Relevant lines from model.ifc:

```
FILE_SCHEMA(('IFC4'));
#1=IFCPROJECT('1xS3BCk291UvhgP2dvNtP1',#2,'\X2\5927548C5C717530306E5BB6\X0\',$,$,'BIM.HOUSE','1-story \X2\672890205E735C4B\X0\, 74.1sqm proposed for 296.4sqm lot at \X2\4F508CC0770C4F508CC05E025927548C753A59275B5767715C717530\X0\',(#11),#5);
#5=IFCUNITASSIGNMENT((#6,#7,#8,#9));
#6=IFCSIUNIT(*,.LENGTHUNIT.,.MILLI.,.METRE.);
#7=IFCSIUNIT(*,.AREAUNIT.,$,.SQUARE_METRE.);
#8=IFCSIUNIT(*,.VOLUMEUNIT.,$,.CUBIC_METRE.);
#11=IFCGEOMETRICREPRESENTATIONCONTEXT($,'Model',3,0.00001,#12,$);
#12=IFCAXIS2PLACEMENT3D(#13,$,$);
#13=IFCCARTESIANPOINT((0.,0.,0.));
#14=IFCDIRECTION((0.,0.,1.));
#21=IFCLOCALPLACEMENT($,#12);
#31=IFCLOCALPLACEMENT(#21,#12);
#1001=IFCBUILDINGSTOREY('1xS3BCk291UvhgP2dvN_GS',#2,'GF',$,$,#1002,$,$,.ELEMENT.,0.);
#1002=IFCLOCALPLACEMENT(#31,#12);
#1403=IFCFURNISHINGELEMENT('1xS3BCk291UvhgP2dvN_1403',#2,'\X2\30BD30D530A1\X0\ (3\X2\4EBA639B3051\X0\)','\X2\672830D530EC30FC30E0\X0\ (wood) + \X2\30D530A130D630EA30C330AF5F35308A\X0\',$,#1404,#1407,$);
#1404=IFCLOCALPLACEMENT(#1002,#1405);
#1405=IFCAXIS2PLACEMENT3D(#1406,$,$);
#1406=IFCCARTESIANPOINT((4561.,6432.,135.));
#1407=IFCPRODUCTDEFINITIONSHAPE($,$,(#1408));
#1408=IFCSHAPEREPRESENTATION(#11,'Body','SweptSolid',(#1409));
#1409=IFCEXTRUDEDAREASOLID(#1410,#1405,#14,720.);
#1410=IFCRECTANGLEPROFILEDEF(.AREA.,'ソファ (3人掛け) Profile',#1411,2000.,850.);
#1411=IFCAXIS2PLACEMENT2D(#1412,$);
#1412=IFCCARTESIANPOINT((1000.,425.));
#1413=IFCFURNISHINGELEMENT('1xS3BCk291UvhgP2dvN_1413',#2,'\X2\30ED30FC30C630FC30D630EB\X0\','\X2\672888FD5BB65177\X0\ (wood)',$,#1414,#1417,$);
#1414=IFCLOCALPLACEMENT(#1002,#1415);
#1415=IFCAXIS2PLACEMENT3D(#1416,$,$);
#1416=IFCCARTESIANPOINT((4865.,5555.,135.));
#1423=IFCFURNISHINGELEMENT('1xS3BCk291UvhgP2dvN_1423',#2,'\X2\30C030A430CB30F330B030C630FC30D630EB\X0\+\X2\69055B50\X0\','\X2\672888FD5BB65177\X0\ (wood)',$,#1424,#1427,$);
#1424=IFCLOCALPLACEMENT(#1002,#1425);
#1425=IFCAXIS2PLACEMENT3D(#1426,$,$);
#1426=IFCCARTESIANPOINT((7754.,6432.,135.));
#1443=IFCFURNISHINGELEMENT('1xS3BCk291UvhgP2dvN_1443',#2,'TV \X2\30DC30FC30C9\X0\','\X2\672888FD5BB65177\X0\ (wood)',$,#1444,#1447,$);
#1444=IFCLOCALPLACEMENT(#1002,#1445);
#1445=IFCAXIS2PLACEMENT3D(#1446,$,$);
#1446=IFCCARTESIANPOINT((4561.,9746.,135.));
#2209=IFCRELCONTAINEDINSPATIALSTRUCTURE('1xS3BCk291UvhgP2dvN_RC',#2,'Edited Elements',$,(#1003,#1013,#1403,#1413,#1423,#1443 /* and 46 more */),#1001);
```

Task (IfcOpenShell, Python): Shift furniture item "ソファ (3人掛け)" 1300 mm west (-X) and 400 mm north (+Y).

```python
import ifcopenshell
import ifcopenshell.api.geometry
import ifcopenshell.util.placement
import ifcopenshell.util.unit

model = ifcopenshell.open("model.ifc")
unit_scale = ifcopenshell.util.unit.calculate_unit_scale(model)

item = model.by_id(1403)
matrix = ifcopenshell.util.placement.get_local_placement(item.ObjectPlacement)
matrix[0, 3] -= 1.3 / unit_scale
matrix[1, 3] += 0.4 / unit_scale
ifcopenshell.api.geometry.edit_object_placement(model, product=item, matrix=matrix, is_si=False)

print(ifcopenshell.util.placement.get_local_placement(item.ObjectPlacement).round(3) + 0.0)

model.write("model-out.ifc")
```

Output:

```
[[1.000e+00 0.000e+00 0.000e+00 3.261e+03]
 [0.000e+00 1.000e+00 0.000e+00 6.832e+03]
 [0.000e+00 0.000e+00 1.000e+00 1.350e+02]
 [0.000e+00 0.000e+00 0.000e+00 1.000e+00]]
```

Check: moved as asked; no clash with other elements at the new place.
